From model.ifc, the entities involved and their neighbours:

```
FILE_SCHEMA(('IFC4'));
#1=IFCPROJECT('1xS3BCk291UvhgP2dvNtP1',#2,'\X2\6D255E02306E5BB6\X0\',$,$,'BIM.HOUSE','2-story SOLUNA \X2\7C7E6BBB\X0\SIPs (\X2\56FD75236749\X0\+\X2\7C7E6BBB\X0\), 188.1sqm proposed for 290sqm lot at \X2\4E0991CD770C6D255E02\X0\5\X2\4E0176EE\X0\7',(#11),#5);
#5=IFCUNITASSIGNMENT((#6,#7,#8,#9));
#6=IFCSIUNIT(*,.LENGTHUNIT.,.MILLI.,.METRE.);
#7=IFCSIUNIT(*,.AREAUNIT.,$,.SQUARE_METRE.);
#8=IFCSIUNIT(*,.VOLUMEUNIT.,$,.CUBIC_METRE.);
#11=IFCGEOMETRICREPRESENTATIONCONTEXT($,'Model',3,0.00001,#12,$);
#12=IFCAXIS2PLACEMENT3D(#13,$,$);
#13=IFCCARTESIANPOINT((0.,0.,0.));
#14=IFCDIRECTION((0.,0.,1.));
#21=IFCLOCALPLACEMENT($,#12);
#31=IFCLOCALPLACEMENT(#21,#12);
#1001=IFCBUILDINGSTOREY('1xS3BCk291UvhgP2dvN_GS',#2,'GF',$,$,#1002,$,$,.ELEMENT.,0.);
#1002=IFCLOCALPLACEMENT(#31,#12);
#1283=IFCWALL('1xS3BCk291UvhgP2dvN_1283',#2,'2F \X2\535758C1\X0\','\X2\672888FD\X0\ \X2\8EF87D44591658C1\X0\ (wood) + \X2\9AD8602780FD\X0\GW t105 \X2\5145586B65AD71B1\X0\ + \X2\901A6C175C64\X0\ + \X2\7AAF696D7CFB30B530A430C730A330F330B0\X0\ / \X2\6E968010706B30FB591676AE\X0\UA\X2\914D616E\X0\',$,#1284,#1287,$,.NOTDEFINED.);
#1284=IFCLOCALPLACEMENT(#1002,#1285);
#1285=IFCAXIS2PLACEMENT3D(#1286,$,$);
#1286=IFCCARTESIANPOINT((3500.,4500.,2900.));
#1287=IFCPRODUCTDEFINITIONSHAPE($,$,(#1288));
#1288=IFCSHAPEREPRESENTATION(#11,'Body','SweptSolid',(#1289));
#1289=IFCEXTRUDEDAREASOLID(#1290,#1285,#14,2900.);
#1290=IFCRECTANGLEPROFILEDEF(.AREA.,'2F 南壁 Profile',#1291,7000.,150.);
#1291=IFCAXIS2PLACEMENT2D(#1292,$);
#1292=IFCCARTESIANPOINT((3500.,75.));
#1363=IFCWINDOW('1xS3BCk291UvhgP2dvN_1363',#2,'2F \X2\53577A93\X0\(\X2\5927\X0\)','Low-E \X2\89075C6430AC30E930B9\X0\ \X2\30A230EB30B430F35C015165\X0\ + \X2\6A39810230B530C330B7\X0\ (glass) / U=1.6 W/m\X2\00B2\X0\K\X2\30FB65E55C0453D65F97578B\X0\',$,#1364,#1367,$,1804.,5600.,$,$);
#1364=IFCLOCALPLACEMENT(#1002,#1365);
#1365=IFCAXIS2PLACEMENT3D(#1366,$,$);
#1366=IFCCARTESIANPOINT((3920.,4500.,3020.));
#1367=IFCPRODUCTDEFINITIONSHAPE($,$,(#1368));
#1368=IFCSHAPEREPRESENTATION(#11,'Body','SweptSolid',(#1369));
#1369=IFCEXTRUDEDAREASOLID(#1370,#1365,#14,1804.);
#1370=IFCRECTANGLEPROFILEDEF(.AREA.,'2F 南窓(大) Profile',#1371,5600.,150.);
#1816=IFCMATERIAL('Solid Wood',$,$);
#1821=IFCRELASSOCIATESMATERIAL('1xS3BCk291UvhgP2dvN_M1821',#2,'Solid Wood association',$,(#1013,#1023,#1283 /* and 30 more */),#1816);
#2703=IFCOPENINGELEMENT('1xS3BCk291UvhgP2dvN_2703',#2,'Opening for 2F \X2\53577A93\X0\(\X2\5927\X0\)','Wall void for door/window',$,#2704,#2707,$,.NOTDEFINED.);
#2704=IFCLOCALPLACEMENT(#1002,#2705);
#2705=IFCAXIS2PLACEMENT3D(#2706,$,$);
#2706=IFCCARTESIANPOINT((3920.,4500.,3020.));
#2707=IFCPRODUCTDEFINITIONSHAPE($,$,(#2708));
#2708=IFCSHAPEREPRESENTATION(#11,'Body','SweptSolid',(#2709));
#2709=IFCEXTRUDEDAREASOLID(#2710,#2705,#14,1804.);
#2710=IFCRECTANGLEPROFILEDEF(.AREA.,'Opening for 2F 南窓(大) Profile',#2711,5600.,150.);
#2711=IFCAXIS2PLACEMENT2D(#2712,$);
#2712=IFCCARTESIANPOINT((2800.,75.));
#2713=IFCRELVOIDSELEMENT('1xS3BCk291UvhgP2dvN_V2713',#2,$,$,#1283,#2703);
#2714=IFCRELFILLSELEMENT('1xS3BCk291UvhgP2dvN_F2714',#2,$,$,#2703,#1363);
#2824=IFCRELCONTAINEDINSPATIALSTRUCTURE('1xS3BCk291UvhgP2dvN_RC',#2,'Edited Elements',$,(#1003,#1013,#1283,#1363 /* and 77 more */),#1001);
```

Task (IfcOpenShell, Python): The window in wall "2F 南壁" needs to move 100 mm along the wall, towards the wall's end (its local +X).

```python
import ifcopenshell
import ifcopenshell.api.geometry
import ifcopenshell.util.placement
import ifcopenshell.util.unit

model = ifcopenshell.open("model.ifc")
unit_scale = ifcopenshell.util.unit.calculate_unit_scale(model)

window = model.by_guid("1xS3BCk291UvhgP2dvN_1363")
opening = window.FillsVoids[0].RelatingOpeningElement
wall = opening.VoidsElements[0].RelatingBuildingElement

wall_matrix = ifcopenshell.util.placement.get_local_placement(wall.ObjectPlacement)
shift = wall_matrix[:3, 0] * 0.1 / unit_scale
before = ifcopenshell.util.placement.get_local_placement(window.ObjectPlacement)[:3, 3].copy()

# The window is not placed relative to its opening, so move both.
for product in (opening, window):
    matrix = ifcopenshell.util.placement.get_local_placement(product.ObjectPlacement)
    matrix[:3, 3] += shift
    ifcopenshell.api.geometry.edit_object_placement(model, product=product, matrix=matrix, is_si=False)

after = ifcopenshell.util.placement.get_local_placement(window.ObjectPlacement)[:3, 3]
print("window moved by", (after - before).round(3) + 0.0)

model.write("model_rev.ifc")
```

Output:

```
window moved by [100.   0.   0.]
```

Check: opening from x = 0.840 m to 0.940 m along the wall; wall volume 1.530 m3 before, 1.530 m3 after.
